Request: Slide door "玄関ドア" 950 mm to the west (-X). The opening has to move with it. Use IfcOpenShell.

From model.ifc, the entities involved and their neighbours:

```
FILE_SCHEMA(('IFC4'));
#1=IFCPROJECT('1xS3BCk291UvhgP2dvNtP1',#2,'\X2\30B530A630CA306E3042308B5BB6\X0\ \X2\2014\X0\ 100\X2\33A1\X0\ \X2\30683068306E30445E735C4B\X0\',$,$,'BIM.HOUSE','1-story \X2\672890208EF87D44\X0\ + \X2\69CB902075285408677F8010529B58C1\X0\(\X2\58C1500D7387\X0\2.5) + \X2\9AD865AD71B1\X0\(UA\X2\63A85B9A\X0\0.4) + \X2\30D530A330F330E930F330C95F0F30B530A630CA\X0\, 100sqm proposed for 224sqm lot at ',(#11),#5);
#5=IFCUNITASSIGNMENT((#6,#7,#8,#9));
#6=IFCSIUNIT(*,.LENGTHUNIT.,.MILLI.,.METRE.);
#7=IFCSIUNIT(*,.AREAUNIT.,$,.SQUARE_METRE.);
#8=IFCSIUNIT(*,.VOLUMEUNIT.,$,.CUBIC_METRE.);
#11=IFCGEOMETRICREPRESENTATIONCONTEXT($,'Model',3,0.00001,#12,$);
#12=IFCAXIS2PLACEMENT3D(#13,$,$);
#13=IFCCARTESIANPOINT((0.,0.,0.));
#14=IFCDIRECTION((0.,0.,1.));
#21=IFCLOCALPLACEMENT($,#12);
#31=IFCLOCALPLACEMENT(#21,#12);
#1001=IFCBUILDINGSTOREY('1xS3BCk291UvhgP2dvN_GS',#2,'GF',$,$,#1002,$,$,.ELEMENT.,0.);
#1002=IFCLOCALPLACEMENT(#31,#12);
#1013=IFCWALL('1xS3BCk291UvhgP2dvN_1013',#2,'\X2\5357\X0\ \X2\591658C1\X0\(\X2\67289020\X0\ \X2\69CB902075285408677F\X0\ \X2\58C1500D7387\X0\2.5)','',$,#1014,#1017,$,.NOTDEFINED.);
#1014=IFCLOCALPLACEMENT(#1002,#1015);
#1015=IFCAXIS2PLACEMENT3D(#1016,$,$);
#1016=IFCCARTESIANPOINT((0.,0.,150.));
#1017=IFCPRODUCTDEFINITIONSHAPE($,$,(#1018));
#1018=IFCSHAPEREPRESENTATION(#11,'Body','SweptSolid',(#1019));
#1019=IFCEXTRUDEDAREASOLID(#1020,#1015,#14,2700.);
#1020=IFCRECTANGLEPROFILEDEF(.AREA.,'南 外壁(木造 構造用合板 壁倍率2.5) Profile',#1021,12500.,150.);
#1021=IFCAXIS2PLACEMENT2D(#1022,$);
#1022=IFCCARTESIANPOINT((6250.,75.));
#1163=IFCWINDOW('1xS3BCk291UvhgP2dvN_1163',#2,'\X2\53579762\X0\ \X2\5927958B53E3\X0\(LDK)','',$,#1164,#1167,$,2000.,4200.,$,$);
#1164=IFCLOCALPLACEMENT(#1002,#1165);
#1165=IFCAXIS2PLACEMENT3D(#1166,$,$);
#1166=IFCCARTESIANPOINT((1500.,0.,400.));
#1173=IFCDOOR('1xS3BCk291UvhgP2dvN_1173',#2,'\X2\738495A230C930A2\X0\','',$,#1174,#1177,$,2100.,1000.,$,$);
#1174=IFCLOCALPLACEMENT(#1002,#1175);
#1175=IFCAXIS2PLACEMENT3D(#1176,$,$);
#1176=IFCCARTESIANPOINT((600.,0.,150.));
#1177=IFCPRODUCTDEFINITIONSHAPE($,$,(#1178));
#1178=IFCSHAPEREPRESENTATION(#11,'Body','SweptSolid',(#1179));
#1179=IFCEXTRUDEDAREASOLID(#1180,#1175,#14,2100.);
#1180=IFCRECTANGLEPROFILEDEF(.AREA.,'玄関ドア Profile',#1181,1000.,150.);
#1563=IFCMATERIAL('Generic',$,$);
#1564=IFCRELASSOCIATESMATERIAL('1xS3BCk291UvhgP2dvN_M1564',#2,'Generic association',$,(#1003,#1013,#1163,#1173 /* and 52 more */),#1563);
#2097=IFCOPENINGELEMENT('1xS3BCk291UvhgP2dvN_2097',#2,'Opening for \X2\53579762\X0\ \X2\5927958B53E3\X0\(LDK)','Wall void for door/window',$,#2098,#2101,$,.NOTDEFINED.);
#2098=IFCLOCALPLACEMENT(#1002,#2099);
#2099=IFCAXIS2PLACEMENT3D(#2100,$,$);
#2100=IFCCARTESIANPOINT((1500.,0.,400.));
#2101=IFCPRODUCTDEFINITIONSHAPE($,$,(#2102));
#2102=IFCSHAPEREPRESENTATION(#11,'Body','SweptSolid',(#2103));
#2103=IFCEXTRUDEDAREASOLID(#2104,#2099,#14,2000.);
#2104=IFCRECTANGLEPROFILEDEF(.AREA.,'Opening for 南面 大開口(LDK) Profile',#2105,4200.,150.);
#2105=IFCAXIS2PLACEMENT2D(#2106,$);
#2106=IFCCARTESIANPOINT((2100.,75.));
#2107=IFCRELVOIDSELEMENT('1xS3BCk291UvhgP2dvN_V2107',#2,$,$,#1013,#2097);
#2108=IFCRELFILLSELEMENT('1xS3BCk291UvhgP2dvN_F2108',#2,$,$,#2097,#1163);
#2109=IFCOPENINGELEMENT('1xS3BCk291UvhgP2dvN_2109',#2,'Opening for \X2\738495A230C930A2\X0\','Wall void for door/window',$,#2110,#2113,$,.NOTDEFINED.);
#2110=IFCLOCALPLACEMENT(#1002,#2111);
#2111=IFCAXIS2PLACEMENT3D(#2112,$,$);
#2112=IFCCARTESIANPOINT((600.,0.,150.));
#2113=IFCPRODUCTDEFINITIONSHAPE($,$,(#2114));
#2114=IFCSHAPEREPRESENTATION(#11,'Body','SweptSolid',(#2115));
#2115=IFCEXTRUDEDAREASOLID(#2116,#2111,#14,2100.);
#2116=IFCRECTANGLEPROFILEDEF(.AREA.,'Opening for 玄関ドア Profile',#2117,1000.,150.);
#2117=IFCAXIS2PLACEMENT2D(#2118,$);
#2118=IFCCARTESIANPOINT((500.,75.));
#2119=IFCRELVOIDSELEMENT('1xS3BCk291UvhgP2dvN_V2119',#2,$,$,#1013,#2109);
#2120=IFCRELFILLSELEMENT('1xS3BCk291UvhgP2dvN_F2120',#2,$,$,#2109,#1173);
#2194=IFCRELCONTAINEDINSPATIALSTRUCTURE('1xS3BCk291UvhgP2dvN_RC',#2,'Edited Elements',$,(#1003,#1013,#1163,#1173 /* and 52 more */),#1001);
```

```python
import ifcopenshell
import ifcopenshell.api.geometry
import ifcopenshell.util.placement
import ifcopenshell.util.unit

model = ifcopenshell.open("model.ifc")
unit_scale = ifcopenshell.util.unit.calculate_unit_scale(model)

door = model.by_guid("1xS3BCk291UvhgP2dvN_1173")
opening = door.FillsVoids[0].RelatingOpeningElement
wall = opening.VoidsElements[0].RelatingBuildingElement

wall_matrix = ifcopenshell.util.placement.get_local_placement(wall.ObjectPlacement)
shift = wall_matrix[:3, 0] * -0.95 / unit_scale
before = ifcopenshell.util.placement.get_local_placement(door.ObjectPlacement)[:3, 3].copy()

# The door is not placed relative to its opening, so move both.
for product in (opening, door):
    matrix = ifcopenshell.util.placement.get_local_placement(product.ObjectPlacement)
    matrix[:3, 3] += shift
    ifcopenshell.api.geometry.edit_object_placement(model, product=product, matrix=matrix, is_si=False)

after = ifcopenshell.util.placement.get_local_placement(door.ObjectPlacement)[:3, 3]
print("door moved by", (after - before).round(3) + 0.0)

model.write("model_v2.ifc")
```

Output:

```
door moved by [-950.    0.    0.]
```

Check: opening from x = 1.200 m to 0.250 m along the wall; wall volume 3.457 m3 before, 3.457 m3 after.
